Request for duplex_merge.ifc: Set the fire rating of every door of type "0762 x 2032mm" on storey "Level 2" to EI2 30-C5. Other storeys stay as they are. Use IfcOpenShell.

First a look at what the model holds.

```python
import ifcopenshell
import ifcopenshell.util.element

model = ifcopenshell.open("duplex_merge.ifc")
print(model.schema)
storey = next(s for s in model.by_type("IfcBuildingStorey") if s.Name == "Level 2")
doors = [e for e in ifcopenshell.util.element.get_decomposition(storey) if e.is_a("IfcDoor")]
seen = {}
for e in doors:
    element_type = ifcopenshell.util.element.get_type(e)
    key = (element_type.Name if element_type != e and element_type else None, ifcopenshell.util.element.get_pset(e, "Pset_DoorCommon", "FireRating"))
    seen[key] = seen.get(key, 0) + 1
for (name, value), count in sorted(seen.items(), key=str):
    print(count, "x", name, "|", value)
```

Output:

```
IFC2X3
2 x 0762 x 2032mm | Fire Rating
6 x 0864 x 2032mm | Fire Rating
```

```python
import ifcopenshell
import ifcopenshell.api.pset
import ifcopenshell.util.element

model = ifcopenshell.open("duplex_merge.ifc")

storey = next(s for s in model.by_type("IfcBuildingStorey") if s.Name == "Level 2")
doors = [e for e in ifcopenshell.util.element.get_decomposition(storey) if e.is_a("IfcDoor")]

count = 0
for e in doors:
    element_type = ifcopenshell.util.element.get_type(e)
    if element_type in (None, e) or element_type.Name != "0762 x 2032mm":
        continue
    # add_pset returns the element's existing set when there is one.
    pset = ifcopenshell.api.pset.add_pset(model, product=e, name="Pset_DoorCommon")
    ifcopenshell.api.pset.edit_pset(model, pset=pset, properties={"FireRating": "EI2 30-C5"})
    count += 1

print(count, "doors updated")

model.write("duplex_merge_v2.ifc")
```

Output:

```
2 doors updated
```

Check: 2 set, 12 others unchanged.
